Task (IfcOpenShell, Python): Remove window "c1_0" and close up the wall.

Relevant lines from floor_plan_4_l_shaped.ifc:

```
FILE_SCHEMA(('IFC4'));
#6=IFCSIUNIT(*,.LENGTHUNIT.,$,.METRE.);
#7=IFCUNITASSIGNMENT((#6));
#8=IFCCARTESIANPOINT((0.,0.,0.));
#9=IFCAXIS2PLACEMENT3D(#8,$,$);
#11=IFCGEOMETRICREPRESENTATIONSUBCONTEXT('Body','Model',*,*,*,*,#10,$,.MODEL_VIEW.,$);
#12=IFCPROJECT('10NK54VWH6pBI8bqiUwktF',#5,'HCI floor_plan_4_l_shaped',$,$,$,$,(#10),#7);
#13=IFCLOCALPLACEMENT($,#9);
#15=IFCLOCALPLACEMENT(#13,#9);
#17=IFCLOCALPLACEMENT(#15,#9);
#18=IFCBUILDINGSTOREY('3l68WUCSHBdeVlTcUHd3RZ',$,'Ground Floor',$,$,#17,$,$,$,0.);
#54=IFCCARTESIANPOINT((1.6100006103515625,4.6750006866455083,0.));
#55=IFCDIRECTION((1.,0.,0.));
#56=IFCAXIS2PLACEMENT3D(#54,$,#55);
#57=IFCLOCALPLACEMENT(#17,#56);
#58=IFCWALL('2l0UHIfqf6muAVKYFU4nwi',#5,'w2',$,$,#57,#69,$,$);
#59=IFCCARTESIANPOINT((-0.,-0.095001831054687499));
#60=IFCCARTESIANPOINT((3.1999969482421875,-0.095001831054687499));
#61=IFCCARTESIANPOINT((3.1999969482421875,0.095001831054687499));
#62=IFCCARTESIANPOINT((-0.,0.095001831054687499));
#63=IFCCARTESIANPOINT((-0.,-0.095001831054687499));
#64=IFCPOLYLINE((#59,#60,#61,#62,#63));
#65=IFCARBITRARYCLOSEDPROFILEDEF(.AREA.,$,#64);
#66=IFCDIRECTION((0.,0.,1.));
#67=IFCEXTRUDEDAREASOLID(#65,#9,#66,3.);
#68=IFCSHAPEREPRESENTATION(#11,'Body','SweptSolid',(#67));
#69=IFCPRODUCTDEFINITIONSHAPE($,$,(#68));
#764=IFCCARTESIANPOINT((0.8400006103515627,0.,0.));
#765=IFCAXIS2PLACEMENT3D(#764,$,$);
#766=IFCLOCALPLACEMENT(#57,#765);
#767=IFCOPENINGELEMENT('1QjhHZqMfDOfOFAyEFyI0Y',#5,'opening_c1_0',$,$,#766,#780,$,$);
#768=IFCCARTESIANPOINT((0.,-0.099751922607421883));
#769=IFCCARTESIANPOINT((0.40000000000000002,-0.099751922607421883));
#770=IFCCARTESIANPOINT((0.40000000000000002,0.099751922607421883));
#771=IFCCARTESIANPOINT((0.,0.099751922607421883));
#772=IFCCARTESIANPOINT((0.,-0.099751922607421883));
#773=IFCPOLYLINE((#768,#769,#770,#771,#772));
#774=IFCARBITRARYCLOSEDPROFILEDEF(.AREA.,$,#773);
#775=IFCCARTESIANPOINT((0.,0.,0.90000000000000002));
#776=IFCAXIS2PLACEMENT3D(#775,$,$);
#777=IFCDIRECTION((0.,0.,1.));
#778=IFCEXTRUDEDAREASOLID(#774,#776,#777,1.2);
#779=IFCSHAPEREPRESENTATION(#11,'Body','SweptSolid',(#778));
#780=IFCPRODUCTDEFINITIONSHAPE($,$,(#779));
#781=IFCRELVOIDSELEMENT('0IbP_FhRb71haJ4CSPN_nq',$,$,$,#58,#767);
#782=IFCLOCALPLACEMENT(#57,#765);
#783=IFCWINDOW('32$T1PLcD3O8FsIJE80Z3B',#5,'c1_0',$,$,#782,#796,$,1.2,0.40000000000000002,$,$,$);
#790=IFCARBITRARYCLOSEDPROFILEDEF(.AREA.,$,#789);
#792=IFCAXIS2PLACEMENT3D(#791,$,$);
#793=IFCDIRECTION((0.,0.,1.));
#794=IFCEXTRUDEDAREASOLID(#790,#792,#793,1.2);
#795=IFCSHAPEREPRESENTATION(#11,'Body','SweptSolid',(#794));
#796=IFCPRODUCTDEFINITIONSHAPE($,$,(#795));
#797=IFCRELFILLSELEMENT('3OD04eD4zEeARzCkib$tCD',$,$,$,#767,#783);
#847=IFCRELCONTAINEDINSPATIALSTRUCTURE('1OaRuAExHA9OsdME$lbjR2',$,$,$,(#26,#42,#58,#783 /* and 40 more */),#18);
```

```python
import ifcopenshell
import ifcopenshell.api.feature
import ifcopenshell.api.root
import ifcopenshell.geom
import ifcopenshell.util.shape

model = ifcopenshell.open("floor_plan_4_l_shaped.ifc")
settings = ifcopenshell.geom.settings()


def volume(element):
    """Net volume in cubic metres, openings subtracted."""
    shape = ifcopenshell.geom.create_shape(settings, element)
    return ifcopenshell.util.shape.get_volume(shape.geometry)


window = model.by_id(783)
opening = window.FillsVoids[0].RelatingOpeningElement
wall = opening.VoidsElements[0].RelatingBuildingElement
before = volume(wall)

ifcopenshell.api.root.remove_product(model, product=window)
ifcopenshell.api.feature.remove_feature(model, feature=opening)

after = volume(wall)

print(f"wall volume {before:.3f} -> {after:.3f} m3")

model.write("floor_plan_4_l_shaped-out.ifc")
```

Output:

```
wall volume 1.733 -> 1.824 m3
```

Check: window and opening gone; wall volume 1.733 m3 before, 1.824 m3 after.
